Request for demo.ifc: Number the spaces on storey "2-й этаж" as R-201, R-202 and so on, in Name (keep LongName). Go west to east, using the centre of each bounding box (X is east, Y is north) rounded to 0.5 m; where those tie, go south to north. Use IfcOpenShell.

First a look at what the model holds.

```python
import ifcopenshell
import ifcopenshell.util.element
import ifcopenshell.util.placement

model = ifcopenshell.open("demo.ifc")
print(model.schema)
storey = next(s for s in model.by_type("IfcBuildingStorey") if s.Name == "2-й этаж")
spaces = [e for e in ifcopenshell.util.element.get_decomposition(storey) if e.is_a("IfcSpace")]
for e in sorted(spaces, key=lambda e: e.id()):
    origin = ifcopenshell.util.placement.get_local_placement(e.ObjectPlacement)[:3, 3]
    print(e.id(), e.Name, e.LongName, origin.round(2) + 0.0, sep=" | ")
```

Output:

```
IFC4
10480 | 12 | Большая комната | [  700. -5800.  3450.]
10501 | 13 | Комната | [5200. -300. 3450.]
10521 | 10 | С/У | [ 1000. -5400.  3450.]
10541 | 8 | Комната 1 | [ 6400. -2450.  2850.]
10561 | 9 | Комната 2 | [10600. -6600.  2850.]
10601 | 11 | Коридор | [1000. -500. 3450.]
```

```python
import ifcopenshell
import ifcopenshell.geom
import ifcopenshell.util.element
import ifcopenshell.util.shape

model = ifcopenshell.open("demo.ifc")
settings = ifcopenshell.geom.settings()
settings.set("use-world-coords", True)


def centre(element):
    shape = ifcopenshell.geom.create_shape(settings, element)
    return ifcopenshell.util.shape.get_bbox_centroid(shape.geometry)


storey = next(s for s in model.by_type("IfcBuildingStorey") if s.Name == "2-й этаж")
spaces = [e for e in ifcopenshell.util.element.get_decomposition(storey) if e.is_a("IfcSpace")]

# Insertion points can sit at a corner or the storey origin, so sort by the geometry (in metres).
centres = {e: centre(e) for e in spaces}
spaces.sort(key=lambda e: (round(centres[e][0] / 0.5), centres[e][1]))

for i, e in enumerate(spaces, start=1):
    number = f"R-2{i:02d}"
    e.Name = number
    print(e.id(), number)

model.write("demo_edited.ifc")
```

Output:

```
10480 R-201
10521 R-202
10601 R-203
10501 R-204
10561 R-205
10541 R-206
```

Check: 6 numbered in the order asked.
